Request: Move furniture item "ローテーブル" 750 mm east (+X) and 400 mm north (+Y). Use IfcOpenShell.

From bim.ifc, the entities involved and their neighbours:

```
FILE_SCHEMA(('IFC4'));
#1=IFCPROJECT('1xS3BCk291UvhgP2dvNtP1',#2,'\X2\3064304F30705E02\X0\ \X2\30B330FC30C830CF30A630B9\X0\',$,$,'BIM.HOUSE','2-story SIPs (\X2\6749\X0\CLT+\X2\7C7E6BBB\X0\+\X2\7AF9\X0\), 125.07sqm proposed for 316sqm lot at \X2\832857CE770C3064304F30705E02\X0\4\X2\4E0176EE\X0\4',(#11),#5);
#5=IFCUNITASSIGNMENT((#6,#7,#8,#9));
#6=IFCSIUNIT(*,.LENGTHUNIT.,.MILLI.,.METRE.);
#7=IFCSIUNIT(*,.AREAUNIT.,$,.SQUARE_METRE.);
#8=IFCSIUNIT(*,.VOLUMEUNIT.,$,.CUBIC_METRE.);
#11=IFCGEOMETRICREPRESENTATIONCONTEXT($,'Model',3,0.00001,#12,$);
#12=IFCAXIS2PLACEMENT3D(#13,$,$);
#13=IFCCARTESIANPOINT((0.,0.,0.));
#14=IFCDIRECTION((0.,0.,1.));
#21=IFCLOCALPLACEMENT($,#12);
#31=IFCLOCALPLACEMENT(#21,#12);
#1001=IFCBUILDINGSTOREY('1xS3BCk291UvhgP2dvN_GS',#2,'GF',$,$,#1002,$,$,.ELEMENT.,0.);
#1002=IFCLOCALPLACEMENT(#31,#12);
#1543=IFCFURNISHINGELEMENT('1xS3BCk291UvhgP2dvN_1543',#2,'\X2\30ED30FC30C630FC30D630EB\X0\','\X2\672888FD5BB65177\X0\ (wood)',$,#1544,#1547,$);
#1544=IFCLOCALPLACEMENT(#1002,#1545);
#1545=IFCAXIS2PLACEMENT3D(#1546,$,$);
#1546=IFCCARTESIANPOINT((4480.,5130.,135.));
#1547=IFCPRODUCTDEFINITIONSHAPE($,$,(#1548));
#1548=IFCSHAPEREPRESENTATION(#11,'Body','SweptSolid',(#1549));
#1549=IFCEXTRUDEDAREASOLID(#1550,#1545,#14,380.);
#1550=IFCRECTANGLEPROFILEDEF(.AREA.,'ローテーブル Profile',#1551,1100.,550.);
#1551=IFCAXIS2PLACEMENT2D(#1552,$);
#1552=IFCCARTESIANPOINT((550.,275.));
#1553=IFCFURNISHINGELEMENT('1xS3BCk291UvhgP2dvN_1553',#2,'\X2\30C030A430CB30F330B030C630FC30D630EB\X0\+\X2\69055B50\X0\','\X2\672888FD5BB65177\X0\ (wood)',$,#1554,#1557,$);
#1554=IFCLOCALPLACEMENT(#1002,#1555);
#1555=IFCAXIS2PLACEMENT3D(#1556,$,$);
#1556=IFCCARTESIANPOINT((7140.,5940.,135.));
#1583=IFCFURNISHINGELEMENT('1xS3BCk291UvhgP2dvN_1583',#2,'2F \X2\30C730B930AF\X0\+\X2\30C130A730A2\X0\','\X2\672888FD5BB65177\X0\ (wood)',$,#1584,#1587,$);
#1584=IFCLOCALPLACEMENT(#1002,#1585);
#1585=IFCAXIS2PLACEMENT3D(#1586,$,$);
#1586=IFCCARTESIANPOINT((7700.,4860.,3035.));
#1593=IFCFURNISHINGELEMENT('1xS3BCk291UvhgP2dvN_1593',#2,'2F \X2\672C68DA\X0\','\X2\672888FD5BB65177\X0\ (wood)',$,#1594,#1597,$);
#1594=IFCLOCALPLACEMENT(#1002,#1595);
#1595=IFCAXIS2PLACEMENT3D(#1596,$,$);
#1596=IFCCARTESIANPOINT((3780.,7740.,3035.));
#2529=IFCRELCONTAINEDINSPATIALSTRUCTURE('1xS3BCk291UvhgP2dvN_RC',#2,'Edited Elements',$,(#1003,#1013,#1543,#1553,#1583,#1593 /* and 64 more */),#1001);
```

```python
import ifcopenshell
import ifcopenshell.api.geometry
import ifcopenshell.util.placement
import ifcopenshell.util.unit

model = ifcopenshell.open("bim.ifc")
unit_scale = ifcopenshell.util.unit.calculate_unit_scale(model)

item = model.by_guid("1xS3BCk291UvhgP2dvN_1543")
matrix = ifcopenshell.util.placement.get_local_placement(item.ObjectPlacement)
matrix[0, 3] += 0.75 / unit_scale
matrix[1, 3] += 0.4 / unit_scale
ifcopenshell.api.geometry.edit_object_placement(model, product=item, matrix=matrix, is_si=False)

print(ifcopenshell.util.placement.get_local_placement(item.ObjectPlacement).round(3) + 0.0)

model.write("bim_v2.ifc")
```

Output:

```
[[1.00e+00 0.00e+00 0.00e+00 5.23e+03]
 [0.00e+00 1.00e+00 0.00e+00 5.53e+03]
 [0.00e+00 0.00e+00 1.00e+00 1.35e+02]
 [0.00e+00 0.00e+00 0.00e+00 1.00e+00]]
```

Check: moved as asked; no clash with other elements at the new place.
